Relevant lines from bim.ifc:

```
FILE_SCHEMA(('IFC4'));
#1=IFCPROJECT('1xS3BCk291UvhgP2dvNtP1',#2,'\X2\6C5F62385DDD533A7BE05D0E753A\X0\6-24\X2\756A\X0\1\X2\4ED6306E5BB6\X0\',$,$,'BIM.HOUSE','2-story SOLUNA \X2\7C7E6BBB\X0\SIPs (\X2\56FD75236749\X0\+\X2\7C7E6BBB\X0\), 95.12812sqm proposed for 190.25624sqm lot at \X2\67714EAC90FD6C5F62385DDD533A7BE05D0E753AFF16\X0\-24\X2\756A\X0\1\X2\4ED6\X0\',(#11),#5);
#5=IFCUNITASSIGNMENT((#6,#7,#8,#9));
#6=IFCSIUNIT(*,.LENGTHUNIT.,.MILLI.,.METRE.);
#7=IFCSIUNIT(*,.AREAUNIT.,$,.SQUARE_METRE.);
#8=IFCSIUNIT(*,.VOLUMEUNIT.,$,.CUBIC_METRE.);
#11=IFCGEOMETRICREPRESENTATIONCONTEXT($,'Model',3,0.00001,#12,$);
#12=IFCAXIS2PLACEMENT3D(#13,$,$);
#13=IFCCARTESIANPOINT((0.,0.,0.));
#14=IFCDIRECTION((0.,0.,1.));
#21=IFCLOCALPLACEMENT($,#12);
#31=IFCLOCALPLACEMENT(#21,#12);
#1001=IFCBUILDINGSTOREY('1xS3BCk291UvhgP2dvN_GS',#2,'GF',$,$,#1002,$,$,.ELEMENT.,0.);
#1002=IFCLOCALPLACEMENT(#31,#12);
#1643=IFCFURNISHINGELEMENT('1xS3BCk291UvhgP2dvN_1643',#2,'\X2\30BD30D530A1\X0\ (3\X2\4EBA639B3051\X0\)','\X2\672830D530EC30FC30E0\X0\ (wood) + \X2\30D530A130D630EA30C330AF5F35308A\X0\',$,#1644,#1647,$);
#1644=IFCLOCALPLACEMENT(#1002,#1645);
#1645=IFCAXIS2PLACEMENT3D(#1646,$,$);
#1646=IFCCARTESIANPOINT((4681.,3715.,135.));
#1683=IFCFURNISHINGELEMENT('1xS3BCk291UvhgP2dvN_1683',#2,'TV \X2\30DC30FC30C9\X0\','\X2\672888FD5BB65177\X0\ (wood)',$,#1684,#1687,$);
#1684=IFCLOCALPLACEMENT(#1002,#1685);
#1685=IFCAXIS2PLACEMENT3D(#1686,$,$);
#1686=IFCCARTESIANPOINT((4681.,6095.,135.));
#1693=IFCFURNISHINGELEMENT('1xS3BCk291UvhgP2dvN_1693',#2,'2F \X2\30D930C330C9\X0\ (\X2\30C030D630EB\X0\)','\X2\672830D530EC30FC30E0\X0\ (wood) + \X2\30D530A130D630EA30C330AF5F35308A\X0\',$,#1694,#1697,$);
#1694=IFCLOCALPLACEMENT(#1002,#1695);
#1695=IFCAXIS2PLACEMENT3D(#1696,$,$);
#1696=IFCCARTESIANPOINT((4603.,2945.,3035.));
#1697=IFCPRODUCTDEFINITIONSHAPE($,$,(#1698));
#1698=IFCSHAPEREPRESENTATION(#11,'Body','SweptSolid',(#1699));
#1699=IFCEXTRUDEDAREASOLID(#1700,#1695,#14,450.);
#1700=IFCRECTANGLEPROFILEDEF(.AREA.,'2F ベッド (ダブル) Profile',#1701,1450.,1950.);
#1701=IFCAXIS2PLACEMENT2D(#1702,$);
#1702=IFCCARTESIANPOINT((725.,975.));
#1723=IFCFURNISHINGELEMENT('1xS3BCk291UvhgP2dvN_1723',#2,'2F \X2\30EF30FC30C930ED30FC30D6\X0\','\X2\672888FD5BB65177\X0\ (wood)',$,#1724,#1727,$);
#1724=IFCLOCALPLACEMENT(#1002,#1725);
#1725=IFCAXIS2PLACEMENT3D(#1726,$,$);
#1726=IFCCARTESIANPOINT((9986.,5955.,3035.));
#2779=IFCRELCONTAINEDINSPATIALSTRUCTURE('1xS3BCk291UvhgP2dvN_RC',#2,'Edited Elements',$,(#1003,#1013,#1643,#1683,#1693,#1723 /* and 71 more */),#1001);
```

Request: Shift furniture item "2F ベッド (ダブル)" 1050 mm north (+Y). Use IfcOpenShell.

```python
import ifcopenshell
import ifcopenshell.api.geometry
import ifcopenshell.util.placement
import ifcopenshell.util.unit

model = ifcopenshell.open("bim.ifc")
unit_scale = ifcopenshell.util.unit.calculate_unit_scale(model)

item = model.by_guid("1xS3BCk291UvhgP2dvN_1693")
matrix = ifcopenshell.util.placement.get_local_placement(item.ObjectPlacement)
matrix[1, 3] += 1.05 / unit_scale
ifcopenshell.api.geometry.edit_object_placement(model, product=item, matrix=matrix, is_si=False)

print(ifcopenshell.util.placement.get_local_placement(item.ObjectPlacement).round(3) + 0.0)

model.write("bim_rev.ifc")
```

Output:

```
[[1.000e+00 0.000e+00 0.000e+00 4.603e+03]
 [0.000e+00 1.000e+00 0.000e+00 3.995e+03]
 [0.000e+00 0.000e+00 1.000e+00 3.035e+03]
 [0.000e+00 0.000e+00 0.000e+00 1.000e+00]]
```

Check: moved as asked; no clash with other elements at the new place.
